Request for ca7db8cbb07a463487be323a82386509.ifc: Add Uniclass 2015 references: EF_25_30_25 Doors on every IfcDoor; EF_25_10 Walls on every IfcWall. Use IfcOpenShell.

First a look at what the model holds.

```python
import ifcopenshell

model = ifcopenshell.open("ca7db8cbb07a463487be323a82386509.ifc")
print(model.schema)
print("classifications:", [c.Name for c in model.by_type("IfcClassification")])
for ifc_class in ("IfcDoor", "IfcRoof", "IfcStair", "IfcWall", "IfcWindow"):
    print(ifc_class, len(model.by_type(ifc_class)))
```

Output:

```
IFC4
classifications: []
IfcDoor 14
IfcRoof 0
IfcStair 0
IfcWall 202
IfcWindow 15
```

```python
import ifcopenshell
import ifcopenshell.api.classification

model = ifcopenshell.open("ca7db8cbb07a463487be323a82386509.ifc")

system = ifcopenshell.api.classification.add_classification(model, classification="Uniclass 2015")

codes = {
    "IfcDoor": ("EF_25_30_25", "Doors"),
    "IfcWall": ("EF_25_10", "Walls"),
}
for ifc_class, (code, name) in codes.items():
    products = model.by_type(ifc_class)
    ifcopenshell.api.classification.add_reference(
        model, products=products, classification=system, identification=code, name=name
    )
    print(code, len(products))

model.write("ca7db8cbb07a463487be323a82386509_v2.ifc")
```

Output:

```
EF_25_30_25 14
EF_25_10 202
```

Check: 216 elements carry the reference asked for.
